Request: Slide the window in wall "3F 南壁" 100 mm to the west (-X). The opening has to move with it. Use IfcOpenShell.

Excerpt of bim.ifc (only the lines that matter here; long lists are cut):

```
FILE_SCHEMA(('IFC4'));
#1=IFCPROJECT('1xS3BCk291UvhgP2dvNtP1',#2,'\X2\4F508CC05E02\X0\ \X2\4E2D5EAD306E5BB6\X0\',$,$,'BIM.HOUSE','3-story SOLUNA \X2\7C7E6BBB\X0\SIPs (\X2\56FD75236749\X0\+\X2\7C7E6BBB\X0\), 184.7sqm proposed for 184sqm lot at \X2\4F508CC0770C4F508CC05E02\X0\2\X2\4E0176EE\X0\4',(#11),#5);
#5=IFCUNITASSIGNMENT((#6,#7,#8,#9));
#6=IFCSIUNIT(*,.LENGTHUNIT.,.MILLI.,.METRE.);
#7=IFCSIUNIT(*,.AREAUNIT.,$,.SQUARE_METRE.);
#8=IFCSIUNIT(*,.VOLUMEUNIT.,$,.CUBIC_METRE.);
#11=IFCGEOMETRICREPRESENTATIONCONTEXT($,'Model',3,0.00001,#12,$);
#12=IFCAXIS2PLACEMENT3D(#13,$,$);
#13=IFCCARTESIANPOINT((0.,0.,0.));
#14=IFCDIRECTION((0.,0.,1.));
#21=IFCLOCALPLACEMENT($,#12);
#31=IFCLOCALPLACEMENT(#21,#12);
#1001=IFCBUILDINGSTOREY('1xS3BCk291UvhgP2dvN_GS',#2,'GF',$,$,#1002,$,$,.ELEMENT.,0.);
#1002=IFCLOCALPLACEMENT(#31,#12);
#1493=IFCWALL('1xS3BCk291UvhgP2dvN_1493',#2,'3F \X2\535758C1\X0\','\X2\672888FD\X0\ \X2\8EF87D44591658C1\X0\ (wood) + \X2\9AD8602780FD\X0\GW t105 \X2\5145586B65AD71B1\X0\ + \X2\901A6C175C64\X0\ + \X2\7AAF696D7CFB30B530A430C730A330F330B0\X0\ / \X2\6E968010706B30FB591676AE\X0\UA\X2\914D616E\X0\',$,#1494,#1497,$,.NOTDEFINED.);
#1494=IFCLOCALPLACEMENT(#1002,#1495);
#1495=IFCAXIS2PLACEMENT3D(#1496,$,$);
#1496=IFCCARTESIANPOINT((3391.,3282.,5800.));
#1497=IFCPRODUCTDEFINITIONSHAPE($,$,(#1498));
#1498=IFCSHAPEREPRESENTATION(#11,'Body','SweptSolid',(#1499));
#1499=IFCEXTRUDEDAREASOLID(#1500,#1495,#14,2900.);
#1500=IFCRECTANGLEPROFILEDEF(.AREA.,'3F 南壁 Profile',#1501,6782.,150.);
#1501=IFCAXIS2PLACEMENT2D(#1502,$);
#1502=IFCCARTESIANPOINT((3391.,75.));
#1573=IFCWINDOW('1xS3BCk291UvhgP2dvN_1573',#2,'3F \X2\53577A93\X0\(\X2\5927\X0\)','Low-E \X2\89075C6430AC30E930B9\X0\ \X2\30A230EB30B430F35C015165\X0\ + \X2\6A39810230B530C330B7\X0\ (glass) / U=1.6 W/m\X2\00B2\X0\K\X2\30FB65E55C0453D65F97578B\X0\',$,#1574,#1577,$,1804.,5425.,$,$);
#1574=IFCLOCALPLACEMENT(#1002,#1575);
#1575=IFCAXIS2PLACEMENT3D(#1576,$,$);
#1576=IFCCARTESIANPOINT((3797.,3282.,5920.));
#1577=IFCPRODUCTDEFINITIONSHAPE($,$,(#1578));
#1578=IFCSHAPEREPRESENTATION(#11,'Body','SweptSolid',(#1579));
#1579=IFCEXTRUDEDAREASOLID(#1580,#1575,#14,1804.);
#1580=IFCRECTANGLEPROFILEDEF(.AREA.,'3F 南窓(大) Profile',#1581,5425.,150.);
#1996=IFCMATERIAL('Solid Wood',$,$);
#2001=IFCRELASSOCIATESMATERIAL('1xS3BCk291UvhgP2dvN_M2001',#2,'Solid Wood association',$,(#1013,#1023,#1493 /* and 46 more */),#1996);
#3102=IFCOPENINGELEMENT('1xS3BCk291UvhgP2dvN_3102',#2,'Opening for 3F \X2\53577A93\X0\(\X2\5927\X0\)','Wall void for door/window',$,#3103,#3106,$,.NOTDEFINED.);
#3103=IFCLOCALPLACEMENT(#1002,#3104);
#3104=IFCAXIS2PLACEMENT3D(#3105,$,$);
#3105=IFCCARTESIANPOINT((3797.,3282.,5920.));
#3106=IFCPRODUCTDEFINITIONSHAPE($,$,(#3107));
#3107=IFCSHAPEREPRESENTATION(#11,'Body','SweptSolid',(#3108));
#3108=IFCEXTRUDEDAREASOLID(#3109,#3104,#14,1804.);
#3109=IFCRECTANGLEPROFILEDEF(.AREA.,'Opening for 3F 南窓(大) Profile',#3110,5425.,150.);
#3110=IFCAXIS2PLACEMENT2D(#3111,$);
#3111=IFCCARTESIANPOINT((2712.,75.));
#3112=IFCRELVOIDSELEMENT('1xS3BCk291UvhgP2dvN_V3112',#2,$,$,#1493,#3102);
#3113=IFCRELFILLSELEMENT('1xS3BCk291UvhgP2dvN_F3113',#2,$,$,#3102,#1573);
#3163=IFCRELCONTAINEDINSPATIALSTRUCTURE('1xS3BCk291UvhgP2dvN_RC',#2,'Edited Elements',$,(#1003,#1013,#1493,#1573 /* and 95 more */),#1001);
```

```python
import ifcopenshell
import ifcopenshell.api.geometry
import ifcopenshell.util.placement

model = ifcopenshell.open("bim.ifc")

window = model.by_id(1573)
opening = window.FillsVoids[0].RelatingOpeningElement
wall = opening.VoidsElements[0].RelatingBuildingElement

wall_matrix = ifcopenshell.util.placement.get_local_placement(wall.ObjectPlacement)
shift = wall_matrix[:3, 0] * -100.0
before = ifcopenshell.util.placement.get_local_placement(window.ObjectPlacement)[:3, 3].copy()

# The window is not placed relative to its opening, so move both.
for product in (opening, window):
    matrix = ifcopenshell.util.placement.get_local_placement(product.ObjectPlacement)
    matrix[:3, 3] += shift
    ifcopenshell.api.geometry.edit_object_placement(model, product=product, matrix=matrix, is_si=False)

after = ifcopenshell.util.placement.get_local_placement(window.ObjectPlacement)[:3, 3]
print("window moved by", (after - before).round(3) + 0.0)

model.write("bim_v2.ifc")
```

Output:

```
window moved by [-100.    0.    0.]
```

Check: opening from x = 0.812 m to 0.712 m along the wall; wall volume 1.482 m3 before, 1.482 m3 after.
